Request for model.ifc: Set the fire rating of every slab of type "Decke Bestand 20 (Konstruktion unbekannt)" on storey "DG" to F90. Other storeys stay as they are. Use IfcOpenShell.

First a look at what the model holds.

```python
import ifcopenshell
import ifcopenshell.util.element

model = ifcopenshell.open("model.ifc")
print(model.schema)
storey = next(s for s in model.by_type("IfcBuildingStorey") if s.Name == "DG")
slabs = [e for e in ifcopenshell.util.element.get_decomposition(storey) if e.is_a("IfcSlab")]
seen = {}
for e in slabs:
    element_type = ifcopenshell.util.element.get_type(e)
    key = (element_type.Name if element_type != e and element_type else None, ifcopenshell.util.element.get_pset(e, "Pset_SlabCommon", "FireRating"))
    seen[key] = seen.get(key, 0) + 1
for (name, value), count in sorted(seen.items(), key=str):
    print(count, "x", name, "|", value)
```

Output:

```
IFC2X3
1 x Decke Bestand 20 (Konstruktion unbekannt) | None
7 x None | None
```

```python
import ifcopenshell
import ifcopenshell.api.pset
import ifcopenshell.util.element

model = ifcopenshell.open("model.ifc")

storey = next(s for s in model.by_type("IfcBuildingStorey") if s.Name == "DG")
slabs = [e for e in ifcopenshell.util.element.get_decomposition(storey) if e.is_a("IfcSlab")]

count = 0
for e in slabs:
    element_type = ifcopenshell.util.element.get_type(e)
    if element_type in (None, e) or element_type.Name != "Decke Bestand 20 (Konstruktion unbekannt)":
        continue
    # add_pset returns the element's existing set when there is one.
    pset = ifcopenshell.api.pset.add_pset(model, product=e, name="Pset_SlabCommon")
    ifcopenshell.api.pset.edit_pset(model, pset=pset, properties={"FireRating": "F90"})
    count += 1

print(count, "slabs updated")

model.write("model-out.ifc")
```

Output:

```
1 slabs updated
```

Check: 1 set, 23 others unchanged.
